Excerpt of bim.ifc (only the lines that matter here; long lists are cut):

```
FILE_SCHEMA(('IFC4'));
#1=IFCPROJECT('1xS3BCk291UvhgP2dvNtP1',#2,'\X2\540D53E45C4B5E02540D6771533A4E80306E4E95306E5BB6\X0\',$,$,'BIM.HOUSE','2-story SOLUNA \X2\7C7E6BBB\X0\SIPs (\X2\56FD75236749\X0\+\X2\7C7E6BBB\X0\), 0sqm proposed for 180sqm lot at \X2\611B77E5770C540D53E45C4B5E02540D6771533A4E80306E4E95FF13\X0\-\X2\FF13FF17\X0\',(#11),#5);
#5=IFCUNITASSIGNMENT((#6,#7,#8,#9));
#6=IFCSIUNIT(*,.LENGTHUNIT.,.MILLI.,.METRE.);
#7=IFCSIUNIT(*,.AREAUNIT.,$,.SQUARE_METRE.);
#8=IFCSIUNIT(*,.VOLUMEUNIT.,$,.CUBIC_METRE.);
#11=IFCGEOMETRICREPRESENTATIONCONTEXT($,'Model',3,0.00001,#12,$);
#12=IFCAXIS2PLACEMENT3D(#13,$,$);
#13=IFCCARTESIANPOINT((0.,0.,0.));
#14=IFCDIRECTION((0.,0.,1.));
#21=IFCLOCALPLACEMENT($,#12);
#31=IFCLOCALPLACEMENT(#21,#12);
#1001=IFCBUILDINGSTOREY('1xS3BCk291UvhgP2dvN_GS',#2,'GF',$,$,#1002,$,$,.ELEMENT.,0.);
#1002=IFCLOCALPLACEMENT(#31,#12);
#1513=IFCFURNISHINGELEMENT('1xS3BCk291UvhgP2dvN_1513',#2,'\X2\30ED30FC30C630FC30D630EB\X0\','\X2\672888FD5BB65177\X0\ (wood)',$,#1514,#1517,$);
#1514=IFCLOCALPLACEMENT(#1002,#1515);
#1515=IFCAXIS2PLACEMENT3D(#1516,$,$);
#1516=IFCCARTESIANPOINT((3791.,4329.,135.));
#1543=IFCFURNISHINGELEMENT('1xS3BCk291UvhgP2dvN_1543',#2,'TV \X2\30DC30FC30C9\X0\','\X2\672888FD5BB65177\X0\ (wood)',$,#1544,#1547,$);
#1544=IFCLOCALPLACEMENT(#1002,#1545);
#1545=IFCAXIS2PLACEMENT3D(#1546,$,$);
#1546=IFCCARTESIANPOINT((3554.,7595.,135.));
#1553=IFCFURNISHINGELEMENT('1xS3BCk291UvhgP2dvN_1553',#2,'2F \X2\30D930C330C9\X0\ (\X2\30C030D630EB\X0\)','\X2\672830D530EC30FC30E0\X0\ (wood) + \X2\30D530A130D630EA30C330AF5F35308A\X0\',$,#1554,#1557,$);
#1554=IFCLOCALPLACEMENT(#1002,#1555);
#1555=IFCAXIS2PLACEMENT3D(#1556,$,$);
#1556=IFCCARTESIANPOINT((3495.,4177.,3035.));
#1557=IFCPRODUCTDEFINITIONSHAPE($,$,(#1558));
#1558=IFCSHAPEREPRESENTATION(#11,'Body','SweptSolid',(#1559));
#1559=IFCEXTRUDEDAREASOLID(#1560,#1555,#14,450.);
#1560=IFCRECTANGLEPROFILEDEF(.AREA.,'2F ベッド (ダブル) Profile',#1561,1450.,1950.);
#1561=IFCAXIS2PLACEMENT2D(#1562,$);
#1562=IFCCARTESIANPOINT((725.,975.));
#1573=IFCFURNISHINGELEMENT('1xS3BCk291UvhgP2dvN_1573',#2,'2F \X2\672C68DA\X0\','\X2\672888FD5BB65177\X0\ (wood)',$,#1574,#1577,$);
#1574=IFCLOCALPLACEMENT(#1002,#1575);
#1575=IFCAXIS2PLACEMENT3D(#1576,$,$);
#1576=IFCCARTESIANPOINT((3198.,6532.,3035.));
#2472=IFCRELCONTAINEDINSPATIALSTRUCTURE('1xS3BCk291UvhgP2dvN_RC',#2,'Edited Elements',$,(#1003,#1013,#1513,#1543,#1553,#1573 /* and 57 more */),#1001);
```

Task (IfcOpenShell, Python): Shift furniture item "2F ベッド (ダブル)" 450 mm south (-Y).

```python
import ifcopenshell
import ifcopenshell.api.geometry
import ifcopenshell.util.placement

model = ifcopenshell.open("bim.ifc")

item = model.by_guid("1xS3BCk291UvhgP2dvN_1553")
matrix = ifcopenshell.util.placement.get_local_placement(item.ObjectPlacement)
matrix[1, 3] -= 450.0
ifcopenshell.api.geometry.edit_object_placement(model, product=item, matrix=matrix, is_si=False)

print(ifcopenshell.util.placement.get_local_placement(item.ObjectPlacement).round(3) + 0.0)

model.write("bim_v2.ifc")
```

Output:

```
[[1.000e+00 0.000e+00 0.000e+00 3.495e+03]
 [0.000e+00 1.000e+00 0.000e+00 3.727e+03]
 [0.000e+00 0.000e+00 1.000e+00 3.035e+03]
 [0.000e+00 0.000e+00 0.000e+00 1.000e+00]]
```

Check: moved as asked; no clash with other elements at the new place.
